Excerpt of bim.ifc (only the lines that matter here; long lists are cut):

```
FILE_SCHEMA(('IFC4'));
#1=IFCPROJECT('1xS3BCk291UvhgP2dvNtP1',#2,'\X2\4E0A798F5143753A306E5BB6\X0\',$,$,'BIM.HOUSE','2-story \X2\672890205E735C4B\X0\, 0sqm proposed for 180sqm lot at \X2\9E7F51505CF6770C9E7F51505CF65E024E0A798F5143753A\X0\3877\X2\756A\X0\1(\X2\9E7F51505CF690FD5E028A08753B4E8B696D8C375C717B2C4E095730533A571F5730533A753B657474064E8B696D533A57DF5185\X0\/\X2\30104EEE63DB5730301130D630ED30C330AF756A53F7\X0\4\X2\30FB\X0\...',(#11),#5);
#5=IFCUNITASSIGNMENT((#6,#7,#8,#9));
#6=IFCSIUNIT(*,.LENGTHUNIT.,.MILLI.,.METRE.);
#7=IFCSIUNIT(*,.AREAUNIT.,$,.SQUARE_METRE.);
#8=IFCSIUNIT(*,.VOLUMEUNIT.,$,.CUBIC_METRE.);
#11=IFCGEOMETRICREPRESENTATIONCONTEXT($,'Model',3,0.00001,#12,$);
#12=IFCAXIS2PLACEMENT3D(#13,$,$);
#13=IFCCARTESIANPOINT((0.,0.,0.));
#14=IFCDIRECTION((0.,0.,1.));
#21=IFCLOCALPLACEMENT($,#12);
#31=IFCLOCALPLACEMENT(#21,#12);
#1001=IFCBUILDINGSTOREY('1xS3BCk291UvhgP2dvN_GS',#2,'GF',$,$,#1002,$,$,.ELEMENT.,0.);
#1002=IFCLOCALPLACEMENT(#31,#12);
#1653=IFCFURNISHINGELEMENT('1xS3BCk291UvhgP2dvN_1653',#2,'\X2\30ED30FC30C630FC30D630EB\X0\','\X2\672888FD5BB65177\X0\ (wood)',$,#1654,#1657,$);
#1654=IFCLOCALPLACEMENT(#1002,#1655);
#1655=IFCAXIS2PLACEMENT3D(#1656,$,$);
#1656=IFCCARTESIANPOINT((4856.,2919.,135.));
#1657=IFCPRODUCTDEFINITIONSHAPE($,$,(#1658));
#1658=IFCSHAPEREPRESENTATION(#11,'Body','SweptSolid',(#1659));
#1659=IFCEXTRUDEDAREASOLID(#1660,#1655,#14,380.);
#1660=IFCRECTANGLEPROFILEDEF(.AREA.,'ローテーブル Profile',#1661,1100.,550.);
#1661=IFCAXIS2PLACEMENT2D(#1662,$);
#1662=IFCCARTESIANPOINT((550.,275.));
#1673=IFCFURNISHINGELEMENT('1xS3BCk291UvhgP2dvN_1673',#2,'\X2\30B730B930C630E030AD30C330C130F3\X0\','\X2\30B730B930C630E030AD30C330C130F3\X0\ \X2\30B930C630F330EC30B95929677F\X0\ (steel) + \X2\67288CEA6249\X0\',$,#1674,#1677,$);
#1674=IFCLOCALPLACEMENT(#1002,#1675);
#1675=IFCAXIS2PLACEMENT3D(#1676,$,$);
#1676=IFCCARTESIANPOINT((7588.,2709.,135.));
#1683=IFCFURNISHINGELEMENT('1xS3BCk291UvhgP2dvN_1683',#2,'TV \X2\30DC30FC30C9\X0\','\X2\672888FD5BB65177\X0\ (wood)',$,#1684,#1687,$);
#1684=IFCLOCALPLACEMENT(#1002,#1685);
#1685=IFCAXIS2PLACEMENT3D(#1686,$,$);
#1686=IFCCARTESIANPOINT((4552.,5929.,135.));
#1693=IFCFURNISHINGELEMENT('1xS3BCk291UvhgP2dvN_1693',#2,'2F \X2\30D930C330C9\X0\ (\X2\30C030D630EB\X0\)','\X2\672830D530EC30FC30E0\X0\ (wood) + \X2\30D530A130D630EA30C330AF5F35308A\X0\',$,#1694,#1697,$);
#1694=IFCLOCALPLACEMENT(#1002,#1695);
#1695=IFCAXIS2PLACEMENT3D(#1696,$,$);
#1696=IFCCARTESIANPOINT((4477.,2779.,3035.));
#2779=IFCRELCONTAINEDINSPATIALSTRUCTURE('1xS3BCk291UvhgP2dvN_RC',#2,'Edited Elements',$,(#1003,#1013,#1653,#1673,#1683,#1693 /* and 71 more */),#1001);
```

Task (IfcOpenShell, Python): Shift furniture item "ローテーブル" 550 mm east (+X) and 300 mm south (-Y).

```python
import ifcopenshell
import ifcopenshell.api.geometry
import ifcopenshell.util.placement
import ifcopenshell.util.unit

model = ifcopenshell.open("bim.ifc")
unit_scale = ifcopenshell.util.unit.calculate_unit_scale(model)

item = model.by_guid("1xS3BCk291UvhgP2dvN_1653")
matrix = ifcopenshell.util.placement.get_local_placement(item.ObjectPlacement)
matrix[0, 3] += 0.55 / unit_scale
matrix[1, 3] -= 0.3 / unit_scale
ifcopenshell.api.geometry.edit_object_placement(model, product=item, matrix=matrix, is_si=False)

print(ifcopenshell.util.placement.get_local_placement(item.ObjectPlacement).round(3) + 0.0)

model.write("bim_edited.ifc")
```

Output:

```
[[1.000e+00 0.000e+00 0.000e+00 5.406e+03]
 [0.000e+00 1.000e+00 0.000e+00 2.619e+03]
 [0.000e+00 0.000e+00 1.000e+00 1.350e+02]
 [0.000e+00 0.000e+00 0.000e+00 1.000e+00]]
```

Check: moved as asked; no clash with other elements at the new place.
